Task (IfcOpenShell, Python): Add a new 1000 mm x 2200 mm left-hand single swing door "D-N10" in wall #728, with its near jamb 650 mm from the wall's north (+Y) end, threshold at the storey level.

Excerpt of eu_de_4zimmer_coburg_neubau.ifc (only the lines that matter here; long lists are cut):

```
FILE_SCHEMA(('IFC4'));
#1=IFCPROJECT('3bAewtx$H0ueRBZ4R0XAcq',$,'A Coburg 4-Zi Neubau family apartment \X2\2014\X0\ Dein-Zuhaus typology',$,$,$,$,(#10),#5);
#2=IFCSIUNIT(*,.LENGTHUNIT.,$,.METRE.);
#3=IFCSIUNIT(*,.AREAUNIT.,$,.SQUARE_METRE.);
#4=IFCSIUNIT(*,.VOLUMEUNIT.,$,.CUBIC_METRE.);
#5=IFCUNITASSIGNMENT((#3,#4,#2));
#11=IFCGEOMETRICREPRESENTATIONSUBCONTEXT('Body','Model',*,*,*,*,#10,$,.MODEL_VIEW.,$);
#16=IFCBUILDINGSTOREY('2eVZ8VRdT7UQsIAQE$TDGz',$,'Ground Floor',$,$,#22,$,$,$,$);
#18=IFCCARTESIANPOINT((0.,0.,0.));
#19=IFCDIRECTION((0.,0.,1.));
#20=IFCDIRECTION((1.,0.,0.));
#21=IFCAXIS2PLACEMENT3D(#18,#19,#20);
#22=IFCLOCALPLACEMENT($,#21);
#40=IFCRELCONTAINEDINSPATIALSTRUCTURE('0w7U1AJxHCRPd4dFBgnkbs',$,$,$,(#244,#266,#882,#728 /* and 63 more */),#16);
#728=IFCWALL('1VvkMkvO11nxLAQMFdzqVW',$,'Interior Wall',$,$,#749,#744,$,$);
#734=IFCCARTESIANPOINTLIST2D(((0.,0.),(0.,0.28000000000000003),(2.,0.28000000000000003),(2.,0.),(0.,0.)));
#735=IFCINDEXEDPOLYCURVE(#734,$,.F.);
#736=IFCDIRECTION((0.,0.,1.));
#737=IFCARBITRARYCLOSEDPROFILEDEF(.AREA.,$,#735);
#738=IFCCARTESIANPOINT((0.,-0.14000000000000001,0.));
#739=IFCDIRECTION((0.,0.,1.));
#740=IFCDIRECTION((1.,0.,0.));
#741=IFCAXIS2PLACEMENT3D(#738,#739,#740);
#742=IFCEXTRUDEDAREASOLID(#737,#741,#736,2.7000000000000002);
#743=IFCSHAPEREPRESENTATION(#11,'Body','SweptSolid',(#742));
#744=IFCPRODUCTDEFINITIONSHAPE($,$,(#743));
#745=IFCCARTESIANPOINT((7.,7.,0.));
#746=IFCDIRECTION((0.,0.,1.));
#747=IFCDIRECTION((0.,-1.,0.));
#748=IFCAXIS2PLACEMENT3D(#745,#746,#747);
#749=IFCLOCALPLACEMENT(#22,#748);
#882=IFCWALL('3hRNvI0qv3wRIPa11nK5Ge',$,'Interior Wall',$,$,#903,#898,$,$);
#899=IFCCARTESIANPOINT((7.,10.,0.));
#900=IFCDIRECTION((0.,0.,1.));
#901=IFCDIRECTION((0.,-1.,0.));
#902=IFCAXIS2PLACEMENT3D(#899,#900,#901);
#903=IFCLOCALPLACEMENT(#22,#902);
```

```python
import numpy as np
import ifcopenshell
import ifcopenshell.api.feature
import ifcopenshell.api.geometry
import ifcopenshell.api.root
import ifcopenshell.api.spatial
import ifcopenshell.geom
import ifcopenshell.util.element
import ifcopenshell.util.placement
import ifcopenshell.util.representation
import ifcopenshell.util.shape
import ifcopenshell.util.unit

model = ifcopenshell.open("eu_de_4zimmer_coburg_neubau.ifc")
unit_scale = ifcopenshell.util.unit.calculate_unit_scale(model)
settings = ifcopenshell.geom.settings()


def volume(element):
    """Net volume in cubic metres, openings subtracted."""
    shape = ifcopenshell.geom.create_shape(settings, element)
    return ifcopenshell.util.shape.get_volume(shape.geometry)


wall = model.by_guid("1VvkMkvO11nxLAQMFdzqVW")
storey = ifcopenshell.util.element.get_container(wall, ifc_class="IfcBuildingStorey")
context = ifcopenshell.util.representation.get_context(model, "Model", "Body", "MODEL_VIEW")
before = volume(wall)

width, height, from_end, sill = 1, 2.2, 0.65, 0.0  # metres

# The wall runs along its own X axis, and the end named is its -X end.
wall_shape = ifcopenshell.geom.create_shape(settings, wall)
x, y, z = ifcopenshell.util.shape.get_vertices(wall_shape.geometry).T
start = x.min() + from_end
face, thickness = float(y.min()), float(y.max() - y.min())
wall_matrix = ifcopenshell.util.placement.get_local_placement(wall.ObjectPlacement)
level = ifcopenshell.util.placement.get_local_placement(storey.ObjectPlacement)[2, 3]


def in_wall(x, y):
    """Placement at x, y metres in the wall's axes, at sill height."""
    matrix = wall_matrix.copy()
    matrix[:, 3] = wall_matrix @ np.array([x / unit_scale, y / unit_scale, 0.0, 1.0])
    matrix[2, 3] = level + sill / unit_scale
    return matrix


# Opening: a box that overshoots both wall faces by 50 mm.
opening = ifcopenshell.api.root.create_entity(model, ifc_class="IfcOpeningElement", predefined_type="OPENING")
box = ifcopenshell.api.geometry.add_wall_representation(
    model, context=context, length=width, height=height, thickness=thickness + 0.1
)
ifcopenshell.api.geometry.assign_representation(model, product=opening, representation=box)
ifcopenshell.api.geometry.edit_object_placement(model, product=opening, matrix=in_wall(start, face - 0.05), is_si=False)
ifcopenshell.api.feature.add_feature(model, feature=opening, element=wall)

door = ifcopenshell.api.root.create_entity(model, ifc_class="IfcDoor", name="D-N10", predefined_type="DOOR")
door.OverallWidth, door.OverallHeight = width / unit_scale, height / unit_scale
door.OperationType = "SINGLE_SWING_LEFT"
body = ifcopenshell.api.geometry.add_door_representation(
    model,
    context=context,
    overall_width=door.OverallWidth,
    overall_height=door.OverallHeight,
    operation_type="SINGLE_SWING_LEFT",
    lining_properties={"LiningDepth": thickness / unit_scale, "ThresholdDepth": thickness / unit_scale},
)
ifcopenshell.api.geometry.assign_representation(model, product=door, representation=body)
ifcopenshell.api.spatial.assign_container(model, products=[door], relating_structure=storey)
ifcopenshell.api.feature.add_filling(model, opening=opening, element=door)

# The lining spans the wall, so the door starts at the wall face.
ifcopenshell.api.geometry.edit_object_placement(model, product=door, matrix=in_wall(start, face), is_si=False)

after = volume(wall)

print(f"wall volume {before:.3f} -> {after:.3f} m3")

model.write("eu_de_4zimmer_coburg_neubau_edited.ifc")
```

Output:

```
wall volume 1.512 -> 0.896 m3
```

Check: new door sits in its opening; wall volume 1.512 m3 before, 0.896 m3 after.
